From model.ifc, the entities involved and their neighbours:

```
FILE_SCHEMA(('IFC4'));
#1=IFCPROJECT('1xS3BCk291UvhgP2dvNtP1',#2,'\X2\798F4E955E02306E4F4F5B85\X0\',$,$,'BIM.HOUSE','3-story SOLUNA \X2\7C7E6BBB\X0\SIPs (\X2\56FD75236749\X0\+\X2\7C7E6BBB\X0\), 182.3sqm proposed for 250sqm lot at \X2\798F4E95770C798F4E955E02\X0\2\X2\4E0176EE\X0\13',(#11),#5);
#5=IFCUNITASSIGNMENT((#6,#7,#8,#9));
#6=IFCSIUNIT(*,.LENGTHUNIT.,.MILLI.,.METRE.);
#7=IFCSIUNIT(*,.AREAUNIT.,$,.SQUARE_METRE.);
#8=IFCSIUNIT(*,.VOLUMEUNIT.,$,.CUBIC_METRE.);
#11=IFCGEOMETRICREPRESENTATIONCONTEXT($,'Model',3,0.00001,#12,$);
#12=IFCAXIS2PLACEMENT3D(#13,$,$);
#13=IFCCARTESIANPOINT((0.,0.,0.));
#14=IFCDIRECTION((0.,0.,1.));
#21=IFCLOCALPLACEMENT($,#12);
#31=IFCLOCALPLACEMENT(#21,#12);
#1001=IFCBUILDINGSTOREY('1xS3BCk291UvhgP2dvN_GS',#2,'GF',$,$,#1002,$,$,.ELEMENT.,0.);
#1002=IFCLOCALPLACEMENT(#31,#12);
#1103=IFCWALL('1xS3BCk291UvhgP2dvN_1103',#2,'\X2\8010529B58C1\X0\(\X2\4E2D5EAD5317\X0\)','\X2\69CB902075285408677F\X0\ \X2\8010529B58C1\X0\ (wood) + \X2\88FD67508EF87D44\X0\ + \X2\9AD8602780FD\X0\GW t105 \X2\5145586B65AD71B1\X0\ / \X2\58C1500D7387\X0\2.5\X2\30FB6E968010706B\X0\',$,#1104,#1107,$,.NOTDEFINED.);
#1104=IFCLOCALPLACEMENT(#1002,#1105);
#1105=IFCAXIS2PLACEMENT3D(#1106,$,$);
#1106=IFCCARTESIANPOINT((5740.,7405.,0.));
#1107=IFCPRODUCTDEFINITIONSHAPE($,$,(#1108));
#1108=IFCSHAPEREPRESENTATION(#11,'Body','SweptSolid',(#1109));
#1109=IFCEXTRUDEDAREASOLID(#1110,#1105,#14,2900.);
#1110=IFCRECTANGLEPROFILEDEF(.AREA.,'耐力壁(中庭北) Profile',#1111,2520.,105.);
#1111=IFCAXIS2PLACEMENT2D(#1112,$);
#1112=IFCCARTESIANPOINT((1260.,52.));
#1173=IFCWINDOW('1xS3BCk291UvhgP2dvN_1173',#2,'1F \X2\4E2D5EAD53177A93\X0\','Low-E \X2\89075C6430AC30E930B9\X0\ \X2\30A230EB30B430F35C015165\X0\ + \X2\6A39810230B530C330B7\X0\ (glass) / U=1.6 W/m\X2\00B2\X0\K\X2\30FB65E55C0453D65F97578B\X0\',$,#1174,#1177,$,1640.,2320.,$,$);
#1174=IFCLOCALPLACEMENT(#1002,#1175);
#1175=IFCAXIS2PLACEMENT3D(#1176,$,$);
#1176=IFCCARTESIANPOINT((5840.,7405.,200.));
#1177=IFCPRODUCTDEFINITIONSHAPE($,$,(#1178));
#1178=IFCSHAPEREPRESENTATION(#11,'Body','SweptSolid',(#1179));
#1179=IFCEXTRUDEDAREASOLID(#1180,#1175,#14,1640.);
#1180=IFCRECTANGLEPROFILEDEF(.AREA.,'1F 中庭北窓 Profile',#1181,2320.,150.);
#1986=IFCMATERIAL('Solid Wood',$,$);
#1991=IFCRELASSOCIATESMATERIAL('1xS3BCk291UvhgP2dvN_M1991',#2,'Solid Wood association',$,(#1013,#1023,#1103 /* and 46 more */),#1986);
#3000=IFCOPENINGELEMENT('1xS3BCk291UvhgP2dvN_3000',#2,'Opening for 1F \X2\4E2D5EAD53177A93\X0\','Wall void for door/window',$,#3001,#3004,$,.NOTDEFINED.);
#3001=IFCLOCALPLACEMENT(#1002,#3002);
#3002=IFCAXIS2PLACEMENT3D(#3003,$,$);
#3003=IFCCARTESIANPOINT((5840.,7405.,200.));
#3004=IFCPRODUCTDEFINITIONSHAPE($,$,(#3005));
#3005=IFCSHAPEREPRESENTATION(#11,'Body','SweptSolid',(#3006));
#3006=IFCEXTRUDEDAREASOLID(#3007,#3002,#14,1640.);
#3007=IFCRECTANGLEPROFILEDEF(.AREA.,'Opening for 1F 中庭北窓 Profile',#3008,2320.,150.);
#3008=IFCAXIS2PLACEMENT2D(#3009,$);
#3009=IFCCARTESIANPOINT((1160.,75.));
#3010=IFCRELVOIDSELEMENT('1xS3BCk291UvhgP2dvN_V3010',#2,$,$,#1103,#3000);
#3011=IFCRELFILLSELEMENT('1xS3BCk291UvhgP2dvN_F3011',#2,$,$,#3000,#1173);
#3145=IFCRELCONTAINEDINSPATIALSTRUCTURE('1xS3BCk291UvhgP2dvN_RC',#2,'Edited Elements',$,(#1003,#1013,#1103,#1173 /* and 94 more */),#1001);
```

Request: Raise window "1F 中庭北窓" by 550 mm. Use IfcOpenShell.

```python
import numpy as np
import ifcopenshell
import ifcopenshell.api.geometry
import ifcopenshell.util.placement
import ifcopenshell.util.unit

model = ifcopenshell.open("model.ifc")
unit_scale = ifcopenshell.util.unit.calculate_unit_scale(model)

window = model.by_guid("1xS3BCk291UvhgP2dvN_1173")
opening = window.FillsVoids[0].RelatingOpeningElement
dz = 0.55 / unit_scale

shift = np.array([0.0, 0.0, dz])
# The window is not placed relative to its opening, so move both.
for product in (opening, window):
    matrix = ifcopenshell.util.placement.get_local_placement(product.ObjectPlacement)
    matrix[:3, 3] += shift
    ifcopenshell.api.geometry.edit_object_placement(model, product=product, matrix=matrix, is_si=False)

print(f"moved by {dz * unit_scale:+.3f} m")

model.write("model_edited.ifc")
```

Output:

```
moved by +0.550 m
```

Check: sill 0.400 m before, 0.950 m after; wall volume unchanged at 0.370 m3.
